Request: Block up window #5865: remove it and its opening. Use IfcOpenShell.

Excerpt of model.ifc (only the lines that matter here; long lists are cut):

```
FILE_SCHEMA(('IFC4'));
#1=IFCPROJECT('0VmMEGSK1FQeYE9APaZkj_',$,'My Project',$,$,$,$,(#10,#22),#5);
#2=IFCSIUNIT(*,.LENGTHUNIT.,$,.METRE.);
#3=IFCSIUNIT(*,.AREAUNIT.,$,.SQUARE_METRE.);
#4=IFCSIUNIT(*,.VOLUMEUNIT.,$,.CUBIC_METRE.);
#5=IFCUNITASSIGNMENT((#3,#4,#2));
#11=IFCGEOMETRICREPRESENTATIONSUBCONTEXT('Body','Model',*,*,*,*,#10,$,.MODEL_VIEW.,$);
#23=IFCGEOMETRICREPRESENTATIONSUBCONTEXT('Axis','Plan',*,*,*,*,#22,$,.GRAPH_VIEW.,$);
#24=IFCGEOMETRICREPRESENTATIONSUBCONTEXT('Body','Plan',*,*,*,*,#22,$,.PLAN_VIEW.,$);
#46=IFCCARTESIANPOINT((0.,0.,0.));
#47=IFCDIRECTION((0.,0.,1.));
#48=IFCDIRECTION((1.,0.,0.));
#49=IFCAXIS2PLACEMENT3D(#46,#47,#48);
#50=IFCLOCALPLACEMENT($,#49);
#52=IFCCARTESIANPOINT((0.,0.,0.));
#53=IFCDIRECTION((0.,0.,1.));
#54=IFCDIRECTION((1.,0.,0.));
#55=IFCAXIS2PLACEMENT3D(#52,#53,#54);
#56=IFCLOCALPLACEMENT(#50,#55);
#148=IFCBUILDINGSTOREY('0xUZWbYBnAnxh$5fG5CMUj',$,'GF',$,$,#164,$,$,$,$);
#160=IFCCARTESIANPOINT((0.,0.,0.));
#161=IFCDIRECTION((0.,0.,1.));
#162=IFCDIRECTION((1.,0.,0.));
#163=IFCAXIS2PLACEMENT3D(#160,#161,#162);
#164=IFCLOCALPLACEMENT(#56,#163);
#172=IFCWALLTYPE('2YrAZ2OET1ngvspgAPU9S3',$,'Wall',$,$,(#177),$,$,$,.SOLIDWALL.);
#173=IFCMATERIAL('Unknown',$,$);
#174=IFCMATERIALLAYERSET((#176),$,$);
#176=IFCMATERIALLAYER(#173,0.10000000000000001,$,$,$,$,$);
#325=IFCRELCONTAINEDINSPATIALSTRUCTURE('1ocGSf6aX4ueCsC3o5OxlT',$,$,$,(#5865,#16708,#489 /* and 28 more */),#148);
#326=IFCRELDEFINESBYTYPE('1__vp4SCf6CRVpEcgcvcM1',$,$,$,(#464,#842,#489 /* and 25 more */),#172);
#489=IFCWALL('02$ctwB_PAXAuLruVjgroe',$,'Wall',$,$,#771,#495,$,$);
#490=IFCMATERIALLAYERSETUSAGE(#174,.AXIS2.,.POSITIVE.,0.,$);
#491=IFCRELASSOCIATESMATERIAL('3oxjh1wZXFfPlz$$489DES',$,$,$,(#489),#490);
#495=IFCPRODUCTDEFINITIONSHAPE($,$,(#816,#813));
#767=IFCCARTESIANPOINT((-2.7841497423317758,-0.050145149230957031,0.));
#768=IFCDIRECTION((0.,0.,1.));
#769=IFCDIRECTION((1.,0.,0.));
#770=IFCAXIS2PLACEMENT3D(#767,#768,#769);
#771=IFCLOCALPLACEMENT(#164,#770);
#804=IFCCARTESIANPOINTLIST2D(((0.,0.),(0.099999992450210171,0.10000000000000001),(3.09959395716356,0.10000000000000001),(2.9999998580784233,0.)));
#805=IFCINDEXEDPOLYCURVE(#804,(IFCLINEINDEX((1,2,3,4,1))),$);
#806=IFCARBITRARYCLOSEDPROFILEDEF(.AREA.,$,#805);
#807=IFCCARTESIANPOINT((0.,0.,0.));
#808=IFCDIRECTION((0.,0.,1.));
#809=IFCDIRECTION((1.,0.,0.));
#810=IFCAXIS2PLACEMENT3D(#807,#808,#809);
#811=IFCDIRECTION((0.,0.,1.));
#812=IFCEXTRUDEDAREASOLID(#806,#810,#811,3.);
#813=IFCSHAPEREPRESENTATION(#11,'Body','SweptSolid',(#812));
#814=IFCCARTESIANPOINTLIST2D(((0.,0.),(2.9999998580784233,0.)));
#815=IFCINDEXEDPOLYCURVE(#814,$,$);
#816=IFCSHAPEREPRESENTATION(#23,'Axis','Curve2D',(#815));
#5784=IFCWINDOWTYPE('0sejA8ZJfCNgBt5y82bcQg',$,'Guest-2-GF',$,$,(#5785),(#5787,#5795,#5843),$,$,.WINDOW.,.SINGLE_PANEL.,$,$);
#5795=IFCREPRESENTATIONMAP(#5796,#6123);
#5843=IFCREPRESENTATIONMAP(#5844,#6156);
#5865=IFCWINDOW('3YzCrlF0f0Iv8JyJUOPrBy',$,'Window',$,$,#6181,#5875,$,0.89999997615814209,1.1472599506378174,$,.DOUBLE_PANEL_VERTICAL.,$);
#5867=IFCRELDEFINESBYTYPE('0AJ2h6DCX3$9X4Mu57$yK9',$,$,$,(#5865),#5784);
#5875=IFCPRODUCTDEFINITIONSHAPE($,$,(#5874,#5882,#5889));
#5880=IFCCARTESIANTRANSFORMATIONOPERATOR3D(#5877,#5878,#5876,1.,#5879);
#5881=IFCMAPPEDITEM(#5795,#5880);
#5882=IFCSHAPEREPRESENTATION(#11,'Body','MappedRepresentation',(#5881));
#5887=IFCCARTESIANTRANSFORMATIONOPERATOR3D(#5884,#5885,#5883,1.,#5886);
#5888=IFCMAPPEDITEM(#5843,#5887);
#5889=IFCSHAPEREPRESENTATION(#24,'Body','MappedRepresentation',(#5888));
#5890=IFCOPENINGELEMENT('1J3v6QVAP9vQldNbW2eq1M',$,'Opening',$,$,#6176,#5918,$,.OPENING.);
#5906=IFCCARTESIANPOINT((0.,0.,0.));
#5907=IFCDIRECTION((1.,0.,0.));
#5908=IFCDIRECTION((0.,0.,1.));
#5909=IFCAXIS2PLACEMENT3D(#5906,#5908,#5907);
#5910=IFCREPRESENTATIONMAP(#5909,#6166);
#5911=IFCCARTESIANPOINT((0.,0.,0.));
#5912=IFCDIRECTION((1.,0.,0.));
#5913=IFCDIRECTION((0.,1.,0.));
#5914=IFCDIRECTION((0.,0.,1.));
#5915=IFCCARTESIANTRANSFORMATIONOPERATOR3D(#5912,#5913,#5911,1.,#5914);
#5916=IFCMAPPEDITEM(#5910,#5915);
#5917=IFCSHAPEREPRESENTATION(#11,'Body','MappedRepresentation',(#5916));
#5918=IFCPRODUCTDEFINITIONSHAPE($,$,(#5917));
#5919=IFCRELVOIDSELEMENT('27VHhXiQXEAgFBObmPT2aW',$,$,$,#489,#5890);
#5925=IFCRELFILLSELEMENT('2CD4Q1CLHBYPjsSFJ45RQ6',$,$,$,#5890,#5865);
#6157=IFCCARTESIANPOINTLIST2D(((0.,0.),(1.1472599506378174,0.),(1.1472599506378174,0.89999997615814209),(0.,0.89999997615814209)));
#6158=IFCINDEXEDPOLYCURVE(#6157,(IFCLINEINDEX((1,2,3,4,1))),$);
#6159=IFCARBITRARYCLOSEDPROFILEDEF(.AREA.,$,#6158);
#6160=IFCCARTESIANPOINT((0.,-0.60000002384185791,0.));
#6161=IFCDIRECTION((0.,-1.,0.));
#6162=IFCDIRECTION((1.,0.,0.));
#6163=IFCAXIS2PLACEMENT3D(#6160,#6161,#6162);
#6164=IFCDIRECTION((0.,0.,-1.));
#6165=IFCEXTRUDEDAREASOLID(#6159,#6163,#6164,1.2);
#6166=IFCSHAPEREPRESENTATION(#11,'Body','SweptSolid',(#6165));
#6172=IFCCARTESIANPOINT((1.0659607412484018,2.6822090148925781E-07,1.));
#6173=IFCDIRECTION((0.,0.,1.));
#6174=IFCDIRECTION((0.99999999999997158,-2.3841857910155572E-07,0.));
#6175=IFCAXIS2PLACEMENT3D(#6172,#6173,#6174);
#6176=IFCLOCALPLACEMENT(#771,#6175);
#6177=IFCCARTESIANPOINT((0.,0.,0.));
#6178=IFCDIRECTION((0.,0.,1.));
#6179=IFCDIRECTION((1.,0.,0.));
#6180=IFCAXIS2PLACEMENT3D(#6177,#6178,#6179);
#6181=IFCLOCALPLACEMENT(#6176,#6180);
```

```python
import ifcopenshell
import ifcopenshell.api.feature
import ifcopenshell.api.root
import ifcopenshell.geom
import ifcopenshell.util.shape

model = ifcopenshell.open("model.ifc")
settings = ifcopenshell.geom.settings()


def volume(element):
    """Net volume in cubic metres, openings subtracted."""
    shape = ifcopenshell.geom.create_shape(settings, element)
    return ifcopenshell.util.shape.get_volume(shape.geometry)


window = model.by_guid("3YzCrlF0f0Iv8JyJUOPrBy")
opening = window.FillsVoids[0].RelatingOpeningElement
wall = opening.VoidsElements[0].RelatingBuildingElement
before = volume(wall)

ifcopenshell.api.root.remove_product(model, product=window)
ifcopenshell.api.feature.remove_feature(model, feature=opening)

after = volume(wall)

print(f"wall volume {before:.3f} -> {after:.3f} m3")

model.write("model_edited.ifc")
```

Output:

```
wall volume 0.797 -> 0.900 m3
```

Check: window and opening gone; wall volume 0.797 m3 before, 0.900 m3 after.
